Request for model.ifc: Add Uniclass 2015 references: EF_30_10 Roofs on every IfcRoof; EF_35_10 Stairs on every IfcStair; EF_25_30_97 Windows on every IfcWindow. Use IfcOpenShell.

First a look at what the model holds.

```python
import ifcopenshell

model = ifcopenshell.open("model.ifc")
print(model.schema)
print("classifications:", [c.Name for c in model.by_type("IfcClassification")])
for ifc_class in ("IfcDoor", "IfcRoof", "IfcStair", "IfcWall", "IfcWindow"):
    print(ifc_class, len(model.by_type(ifc_class)))
```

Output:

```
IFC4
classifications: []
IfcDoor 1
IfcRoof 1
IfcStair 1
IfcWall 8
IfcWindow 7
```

```python
import ifcopenshell
import ifcopenshell.api.classification

model = ifcopenshell.open("model.ifc")

system = ifcopenshell.api.classification.add_classification(model, classification="Uniclass 2015")

codes = {
    "IfcRoof": ("EF_30_10", "Roofs"),
    "IfcStair": ("EF_35_10", "Stairs"),
    "IfcWindow": ("EF_25_30_97", "Windows"),
}
for ifc_class, (code, name) in codes.items():
    products = model.by_type(ifc_class)
    ifcopenshell.api.classification.add_reference(
        model, products=products, classification=system, identification=code, name=name
    )
    print(code, len(products))

model.write("model_rev.ifc")
```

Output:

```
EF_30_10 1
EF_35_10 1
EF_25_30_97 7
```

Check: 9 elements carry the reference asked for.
